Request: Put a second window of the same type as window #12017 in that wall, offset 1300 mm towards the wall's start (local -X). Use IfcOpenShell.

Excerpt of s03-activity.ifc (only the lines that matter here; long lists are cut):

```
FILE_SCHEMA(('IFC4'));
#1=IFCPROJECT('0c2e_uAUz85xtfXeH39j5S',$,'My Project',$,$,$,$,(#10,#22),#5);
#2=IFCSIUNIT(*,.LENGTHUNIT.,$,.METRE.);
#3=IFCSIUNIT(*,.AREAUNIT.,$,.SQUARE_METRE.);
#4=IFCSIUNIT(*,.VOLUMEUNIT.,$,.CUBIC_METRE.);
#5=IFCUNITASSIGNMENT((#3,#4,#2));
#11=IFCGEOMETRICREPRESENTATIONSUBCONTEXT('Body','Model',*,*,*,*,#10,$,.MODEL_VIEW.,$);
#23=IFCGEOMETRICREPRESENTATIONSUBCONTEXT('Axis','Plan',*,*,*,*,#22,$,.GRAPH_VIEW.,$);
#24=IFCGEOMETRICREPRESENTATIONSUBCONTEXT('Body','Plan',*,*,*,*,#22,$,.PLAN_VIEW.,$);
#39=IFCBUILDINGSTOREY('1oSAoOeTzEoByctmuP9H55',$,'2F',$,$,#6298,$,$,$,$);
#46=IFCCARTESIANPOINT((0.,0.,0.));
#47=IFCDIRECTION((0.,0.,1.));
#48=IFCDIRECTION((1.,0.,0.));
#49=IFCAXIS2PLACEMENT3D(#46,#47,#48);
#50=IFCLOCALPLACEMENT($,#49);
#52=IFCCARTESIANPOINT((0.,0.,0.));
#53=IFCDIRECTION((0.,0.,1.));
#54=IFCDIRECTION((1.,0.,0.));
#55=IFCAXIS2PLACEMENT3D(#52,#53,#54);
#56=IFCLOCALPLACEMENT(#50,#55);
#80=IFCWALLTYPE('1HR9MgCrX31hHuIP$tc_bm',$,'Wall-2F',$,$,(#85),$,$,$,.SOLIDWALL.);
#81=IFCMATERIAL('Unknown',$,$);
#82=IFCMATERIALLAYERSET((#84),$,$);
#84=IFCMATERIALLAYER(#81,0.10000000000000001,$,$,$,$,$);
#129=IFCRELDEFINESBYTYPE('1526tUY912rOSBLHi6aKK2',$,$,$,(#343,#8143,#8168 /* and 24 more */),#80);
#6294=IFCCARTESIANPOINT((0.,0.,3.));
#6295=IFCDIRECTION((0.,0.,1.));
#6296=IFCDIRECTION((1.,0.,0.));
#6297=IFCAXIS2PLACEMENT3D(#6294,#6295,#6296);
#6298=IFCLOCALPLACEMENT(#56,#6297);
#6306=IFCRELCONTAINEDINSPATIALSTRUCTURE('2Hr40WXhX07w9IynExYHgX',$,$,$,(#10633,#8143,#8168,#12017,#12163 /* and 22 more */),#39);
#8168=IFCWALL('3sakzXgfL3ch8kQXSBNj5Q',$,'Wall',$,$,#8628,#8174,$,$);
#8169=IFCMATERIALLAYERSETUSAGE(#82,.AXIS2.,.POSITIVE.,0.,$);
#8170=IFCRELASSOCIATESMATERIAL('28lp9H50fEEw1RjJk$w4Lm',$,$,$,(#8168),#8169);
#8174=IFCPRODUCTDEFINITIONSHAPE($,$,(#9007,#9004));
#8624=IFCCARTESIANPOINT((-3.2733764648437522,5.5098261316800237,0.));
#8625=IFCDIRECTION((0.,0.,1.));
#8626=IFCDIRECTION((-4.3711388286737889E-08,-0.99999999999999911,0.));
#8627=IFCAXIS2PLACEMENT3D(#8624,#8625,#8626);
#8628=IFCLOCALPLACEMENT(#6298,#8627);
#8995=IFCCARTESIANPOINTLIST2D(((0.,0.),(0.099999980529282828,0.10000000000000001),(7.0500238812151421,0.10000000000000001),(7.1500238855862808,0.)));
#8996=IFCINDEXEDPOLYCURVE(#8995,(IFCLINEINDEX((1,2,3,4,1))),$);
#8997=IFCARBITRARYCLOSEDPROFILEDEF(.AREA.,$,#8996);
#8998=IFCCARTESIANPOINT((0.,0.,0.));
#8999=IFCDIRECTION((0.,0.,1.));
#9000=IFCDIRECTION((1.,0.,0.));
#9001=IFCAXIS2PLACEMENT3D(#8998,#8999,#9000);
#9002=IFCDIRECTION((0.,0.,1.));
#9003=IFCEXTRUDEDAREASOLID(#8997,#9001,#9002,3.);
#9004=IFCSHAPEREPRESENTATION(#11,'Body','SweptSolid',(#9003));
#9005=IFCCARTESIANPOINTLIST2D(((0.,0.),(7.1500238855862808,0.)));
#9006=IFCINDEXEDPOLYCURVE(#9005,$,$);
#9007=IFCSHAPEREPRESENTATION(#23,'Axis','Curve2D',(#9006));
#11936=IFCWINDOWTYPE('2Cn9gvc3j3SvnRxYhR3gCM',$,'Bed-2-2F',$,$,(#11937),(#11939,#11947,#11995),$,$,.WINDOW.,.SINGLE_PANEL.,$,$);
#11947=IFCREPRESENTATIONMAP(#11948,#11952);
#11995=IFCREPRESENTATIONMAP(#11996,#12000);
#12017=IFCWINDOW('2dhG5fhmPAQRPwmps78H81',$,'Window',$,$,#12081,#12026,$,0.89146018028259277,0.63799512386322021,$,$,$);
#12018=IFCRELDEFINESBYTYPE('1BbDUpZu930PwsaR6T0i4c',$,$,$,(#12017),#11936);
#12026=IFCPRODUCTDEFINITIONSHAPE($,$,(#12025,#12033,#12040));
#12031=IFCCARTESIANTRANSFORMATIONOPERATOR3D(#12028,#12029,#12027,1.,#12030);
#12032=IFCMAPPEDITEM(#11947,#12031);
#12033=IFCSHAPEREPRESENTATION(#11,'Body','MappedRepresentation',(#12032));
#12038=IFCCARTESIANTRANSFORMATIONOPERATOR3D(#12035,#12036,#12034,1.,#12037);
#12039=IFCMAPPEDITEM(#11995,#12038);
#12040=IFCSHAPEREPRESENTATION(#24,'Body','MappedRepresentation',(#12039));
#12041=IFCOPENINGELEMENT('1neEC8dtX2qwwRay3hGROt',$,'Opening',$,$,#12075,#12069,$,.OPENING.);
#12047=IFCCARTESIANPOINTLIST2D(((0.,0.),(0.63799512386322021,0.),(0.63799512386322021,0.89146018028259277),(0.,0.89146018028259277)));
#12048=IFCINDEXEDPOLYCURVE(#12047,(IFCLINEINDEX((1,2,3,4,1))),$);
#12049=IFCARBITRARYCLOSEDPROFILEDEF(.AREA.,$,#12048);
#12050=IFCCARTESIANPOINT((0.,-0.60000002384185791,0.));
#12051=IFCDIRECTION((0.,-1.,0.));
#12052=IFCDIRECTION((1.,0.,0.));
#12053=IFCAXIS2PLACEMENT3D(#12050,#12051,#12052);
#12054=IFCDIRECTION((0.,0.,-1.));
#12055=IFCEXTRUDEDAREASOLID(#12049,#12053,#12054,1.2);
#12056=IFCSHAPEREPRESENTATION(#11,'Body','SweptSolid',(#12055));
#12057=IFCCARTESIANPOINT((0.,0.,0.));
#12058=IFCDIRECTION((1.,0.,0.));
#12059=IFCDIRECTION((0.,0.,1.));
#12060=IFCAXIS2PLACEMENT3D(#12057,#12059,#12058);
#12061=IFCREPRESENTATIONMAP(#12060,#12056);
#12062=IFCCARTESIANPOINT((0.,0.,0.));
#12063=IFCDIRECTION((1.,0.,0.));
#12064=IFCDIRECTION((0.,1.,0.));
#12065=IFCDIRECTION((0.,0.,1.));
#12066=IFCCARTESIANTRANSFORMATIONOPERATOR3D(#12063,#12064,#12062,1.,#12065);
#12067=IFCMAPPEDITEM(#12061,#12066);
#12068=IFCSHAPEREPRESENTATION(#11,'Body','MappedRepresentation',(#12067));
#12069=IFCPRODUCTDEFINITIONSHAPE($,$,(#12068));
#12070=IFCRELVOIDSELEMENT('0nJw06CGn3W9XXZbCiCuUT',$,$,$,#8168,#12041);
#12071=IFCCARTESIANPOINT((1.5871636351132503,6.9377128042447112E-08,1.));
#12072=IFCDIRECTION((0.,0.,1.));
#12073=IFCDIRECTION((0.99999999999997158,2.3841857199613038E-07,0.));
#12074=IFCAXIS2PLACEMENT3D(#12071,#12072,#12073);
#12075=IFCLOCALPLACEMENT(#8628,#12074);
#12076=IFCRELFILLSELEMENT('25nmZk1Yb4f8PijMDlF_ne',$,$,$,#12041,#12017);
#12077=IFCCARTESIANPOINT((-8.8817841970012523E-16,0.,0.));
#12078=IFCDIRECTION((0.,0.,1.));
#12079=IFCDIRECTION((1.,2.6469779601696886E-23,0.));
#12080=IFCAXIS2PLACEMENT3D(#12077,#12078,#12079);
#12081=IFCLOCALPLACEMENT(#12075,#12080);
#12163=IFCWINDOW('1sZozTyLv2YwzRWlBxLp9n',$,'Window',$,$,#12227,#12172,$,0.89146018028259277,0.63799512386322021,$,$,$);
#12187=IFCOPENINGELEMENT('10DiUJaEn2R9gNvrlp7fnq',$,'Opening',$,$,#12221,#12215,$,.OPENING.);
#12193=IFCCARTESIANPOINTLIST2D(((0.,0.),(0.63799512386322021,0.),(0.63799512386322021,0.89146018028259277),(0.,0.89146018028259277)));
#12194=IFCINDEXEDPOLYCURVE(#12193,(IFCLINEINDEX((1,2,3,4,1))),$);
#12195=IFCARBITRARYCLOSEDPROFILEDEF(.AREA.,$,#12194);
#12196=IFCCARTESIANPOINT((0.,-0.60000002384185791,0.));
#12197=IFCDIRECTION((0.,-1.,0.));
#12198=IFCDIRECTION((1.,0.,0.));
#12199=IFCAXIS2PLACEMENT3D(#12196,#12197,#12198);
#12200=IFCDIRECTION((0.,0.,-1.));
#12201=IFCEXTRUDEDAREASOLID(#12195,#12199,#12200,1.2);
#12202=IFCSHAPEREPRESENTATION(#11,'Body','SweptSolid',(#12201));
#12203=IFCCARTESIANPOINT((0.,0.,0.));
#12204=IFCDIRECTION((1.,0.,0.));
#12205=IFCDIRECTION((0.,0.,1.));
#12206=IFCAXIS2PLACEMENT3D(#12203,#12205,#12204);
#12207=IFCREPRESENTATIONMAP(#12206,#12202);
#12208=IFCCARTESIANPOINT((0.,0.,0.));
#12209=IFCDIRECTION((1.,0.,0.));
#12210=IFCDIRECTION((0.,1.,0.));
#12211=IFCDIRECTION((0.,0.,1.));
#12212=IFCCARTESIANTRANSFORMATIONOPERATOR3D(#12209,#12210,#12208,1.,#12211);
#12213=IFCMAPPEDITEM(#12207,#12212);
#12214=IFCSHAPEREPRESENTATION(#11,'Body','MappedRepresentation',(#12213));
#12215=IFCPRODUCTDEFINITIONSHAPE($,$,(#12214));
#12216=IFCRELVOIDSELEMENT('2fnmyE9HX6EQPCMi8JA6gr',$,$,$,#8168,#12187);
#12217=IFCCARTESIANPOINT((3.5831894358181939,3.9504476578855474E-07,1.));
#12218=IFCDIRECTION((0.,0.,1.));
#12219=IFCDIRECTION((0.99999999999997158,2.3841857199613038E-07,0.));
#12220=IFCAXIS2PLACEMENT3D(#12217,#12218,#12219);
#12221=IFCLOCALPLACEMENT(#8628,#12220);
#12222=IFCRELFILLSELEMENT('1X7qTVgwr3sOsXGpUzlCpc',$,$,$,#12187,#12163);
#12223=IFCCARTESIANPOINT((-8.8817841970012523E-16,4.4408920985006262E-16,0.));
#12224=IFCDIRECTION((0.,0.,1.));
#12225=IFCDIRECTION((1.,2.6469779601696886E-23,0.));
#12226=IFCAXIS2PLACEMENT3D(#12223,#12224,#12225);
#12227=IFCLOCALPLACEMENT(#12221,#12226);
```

```python
import ifcopenshell
import ifcopenshell.api.feature
import ifcopenshell.api.geometry
import ifcopenshell.api.root
import ifcopenshell.geom
import ifcopenshell.util.element
import ifcopenshell.util.placement
import ifcopenshell.util.shape
import ifcopenshell.util.unit

model = ifcopenshell.open("s03-activity.ifc")
unit_scale = ifcopenshell.util.unit.calculate_unit_scale(model)
settings = ifcopenshell.geom.settings()


def volume(element):
    """Net volume in cubic metres, openings subtracted."""
    shape = ifcopenshell.geom.create_shape(settings, element)
    return ifcopenshell.util.shape.get_volume(shape.geometry)


window = model.by_guid("2dhG5fhmPAQRPwmps78H81")
opening = window.FillsVoids[0].RelatingOpeningElement
wall = opening.VoidsElements[0].RelatingBuildingElement
before = volume(wall)
shift = ifcopenshell.util.placement.get_local_placement(wall.ObjectPlacement)[:3, 0] * -1.3 / unit_scale

# copy_class copies the void relationship, type, container and properties, but no geometry.
new_opening = ifcopenshell.api.root.copy_class(model, product=opening)
new_opening.Representation = ifcopenshell.util.element.copy_deep(
    model, opening.Representation, exclude=["IfcGeometricRepresentationContext", "IfcRepresentationMap"]
)
new_window = ifcopenshell.api.root.copy_class(model, product=window)
new_window.Representation = ifcopenshell.util.element.copy_deep(
    model, window.Representation, exclude=["IfcGeometricRepresentationContext", "IfcRepresentationMap"]
)
ifcopenshell.api.feature.add_filling(model, opening=new_opening, element=new_window)

for old, new in ((opening, new_opening), (window, new_window)):
    matrix = ifcopenshell.util.placement.get_local_placement(old.ObjectPlacement)
    matrix[:3, 3] += shift
    ifcopenshell.api.geometry.edit_object_placement(model, product=new, matrix=matrix, is_si=False)

after = volume(wall)

print(f"wall volume {before:.3f} -> {after:.3f} m3")

model.write("s03-activity_rev.ifc")
```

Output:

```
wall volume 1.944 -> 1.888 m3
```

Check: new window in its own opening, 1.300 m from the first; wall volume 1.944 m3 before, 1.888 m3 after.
